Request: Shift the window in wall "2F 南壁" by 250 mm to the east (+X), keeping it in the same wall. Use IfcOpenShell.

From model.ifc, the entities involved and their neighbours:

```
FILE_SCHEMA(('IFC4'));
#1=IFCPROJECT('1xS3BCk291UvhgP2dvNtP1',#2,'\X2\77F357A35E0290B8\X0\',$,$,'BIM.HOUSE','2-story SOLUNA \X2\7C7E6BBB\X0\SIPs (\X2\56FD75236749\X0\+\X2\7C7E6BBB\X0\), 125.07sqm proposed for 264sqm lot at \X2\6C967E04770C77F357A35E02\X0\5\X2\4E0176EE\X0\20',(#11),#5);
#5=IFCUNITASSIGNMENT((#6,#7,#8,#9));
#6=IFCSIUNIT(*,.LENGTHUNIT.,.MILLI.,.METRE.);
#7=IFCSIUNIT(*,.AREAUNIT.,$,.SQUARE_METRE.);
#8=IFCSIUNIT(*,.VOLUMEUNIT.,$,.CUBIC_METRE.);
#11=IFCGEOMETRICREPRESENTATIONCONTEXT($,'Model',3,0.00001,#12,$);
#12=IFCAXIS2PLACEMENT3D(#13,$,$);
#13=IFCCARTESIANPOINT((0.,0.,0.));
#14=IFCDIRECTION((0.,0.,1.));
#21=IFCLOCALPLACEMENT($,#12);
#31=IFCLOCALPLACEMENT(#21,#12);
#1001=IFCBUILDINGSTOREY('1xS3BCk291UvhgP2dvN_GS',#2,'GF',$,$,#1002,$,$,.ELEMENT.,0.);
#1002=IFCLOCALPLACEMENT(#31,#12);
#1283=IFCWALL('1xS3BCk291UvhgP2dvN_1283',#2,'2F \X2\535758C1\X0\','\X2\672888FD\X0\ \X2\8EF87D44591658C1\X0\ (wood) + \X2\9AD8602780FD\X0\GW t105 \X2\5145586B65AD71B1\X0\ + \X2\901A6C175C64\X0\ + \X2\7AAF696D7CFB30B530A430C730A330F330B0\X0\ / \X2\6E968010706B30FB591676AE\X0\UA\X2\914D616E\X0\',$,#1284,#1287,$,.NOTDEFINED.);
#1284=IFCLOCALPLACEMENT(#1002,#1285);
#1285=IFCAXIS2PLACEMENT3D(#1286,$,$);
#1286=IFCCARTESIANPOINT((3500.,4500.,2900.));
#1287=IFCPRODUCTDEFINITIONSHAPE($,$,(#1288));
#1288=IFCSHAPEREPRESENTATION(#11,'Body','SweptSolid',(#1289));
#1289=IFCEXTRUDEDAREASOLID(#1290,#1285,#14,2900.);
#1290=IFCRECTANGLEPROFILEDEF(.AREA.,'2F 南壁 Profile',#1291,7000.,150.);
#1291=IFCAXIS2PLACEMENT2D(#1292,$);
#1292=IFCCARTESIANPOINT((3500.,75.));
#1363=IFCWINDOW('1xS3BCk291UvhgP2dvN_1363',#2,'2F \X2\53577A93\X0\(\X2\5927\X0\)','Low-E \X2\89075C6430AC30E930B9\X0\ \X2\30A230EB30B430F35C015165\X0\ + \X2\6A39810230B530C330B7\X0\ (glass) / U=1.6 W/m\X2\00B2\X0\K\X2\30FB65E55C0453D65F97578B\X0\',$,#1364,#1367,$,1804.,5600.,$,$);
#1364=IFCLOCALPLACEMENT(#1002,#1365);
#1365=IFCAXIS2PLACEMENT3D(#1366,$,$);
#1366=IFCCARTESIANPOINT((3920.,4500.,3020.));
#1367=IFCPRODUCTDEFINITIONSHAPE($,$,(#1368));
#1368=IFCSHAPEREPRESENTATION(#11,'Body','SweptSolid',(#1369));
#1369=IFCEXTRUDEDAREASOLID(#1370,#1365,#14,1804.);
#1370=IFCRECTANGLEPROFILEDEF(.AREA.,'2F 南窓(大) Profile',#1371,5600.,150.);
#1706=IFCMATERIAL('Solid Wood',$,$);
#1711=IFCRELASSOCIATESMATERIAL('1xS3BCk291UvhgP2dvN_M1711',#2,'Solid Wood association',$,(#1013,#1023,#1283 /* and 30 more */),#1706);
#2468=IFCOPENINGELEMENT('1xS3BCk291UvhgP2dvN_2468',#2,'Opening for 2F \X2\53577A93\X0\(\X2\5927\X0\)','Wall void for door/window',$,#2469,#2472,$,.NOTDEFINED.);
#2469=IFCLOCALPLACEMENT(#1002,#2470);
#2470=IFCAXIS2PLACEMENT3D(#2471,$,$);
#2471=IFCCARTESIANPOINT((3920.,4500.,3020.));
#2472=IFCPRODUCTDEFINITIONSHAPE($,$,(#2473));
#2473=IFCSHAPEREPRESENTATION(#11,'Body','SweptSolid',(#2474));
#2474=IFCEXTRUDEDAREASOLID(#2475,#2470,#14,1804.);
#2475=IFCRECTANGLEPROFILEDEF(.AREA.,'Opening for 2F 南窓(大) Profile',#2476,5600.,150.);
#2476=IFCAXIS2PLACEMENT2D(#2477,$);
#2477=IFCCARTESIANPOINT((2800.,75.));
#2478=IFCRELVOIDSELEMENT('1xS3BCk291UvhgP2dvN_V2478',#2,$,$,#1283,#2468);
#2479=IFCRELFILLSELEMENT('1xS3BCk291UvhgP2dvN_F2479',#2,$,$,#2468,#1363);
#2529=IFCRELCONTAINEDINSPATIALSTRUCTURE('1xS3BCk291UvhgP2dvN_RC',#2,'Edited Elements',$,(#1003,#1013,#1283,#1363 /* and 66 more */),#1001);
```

```python
import ifcopenshell
import ifcopenshell.api.geometry
import ifcopenshell.util.placement

model = ifcopenshell.open("model.ifc")

window = model.by_guid("1xS3BCk291UvhgP2dvN_1363")
opening = window.FillsVoids[0].RelatingOpeningElement
wall = opening.VoidsElements[0].RelatingBuildingElement

wall_matrix = ifcopenshell.util.placement.get_local_placement(wall.ObjectPlacement)
shift = wall_matrix[:3, 0] * 250.0
before = ifcopenshell.util.placement.get_local_placement(window.ObjectPlacement)[:3, 3].copy()

# The window is not placed relative to its opening, so move both.
for product in (opening, window):
    matrix = ifcopenshell.util.placement.get_local_placement(product.ObjectPlacement)
    matrix[:3, 3] += shift
    ifcopenshell.api.geometry.edit_object_placement(model, product=product, matrix=matrix, is_si=False)

after = ifcopenshell.util.placement.get_local_placement(window.ObjectPlacement)[:3, 3]
print("window moved by", (after - before).round(3) + 0.0)

model.write("model_v2.ifc")
```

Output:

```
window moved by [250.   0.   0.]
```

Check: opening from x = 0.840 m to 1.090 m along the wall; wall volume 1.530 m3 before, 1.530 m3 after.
